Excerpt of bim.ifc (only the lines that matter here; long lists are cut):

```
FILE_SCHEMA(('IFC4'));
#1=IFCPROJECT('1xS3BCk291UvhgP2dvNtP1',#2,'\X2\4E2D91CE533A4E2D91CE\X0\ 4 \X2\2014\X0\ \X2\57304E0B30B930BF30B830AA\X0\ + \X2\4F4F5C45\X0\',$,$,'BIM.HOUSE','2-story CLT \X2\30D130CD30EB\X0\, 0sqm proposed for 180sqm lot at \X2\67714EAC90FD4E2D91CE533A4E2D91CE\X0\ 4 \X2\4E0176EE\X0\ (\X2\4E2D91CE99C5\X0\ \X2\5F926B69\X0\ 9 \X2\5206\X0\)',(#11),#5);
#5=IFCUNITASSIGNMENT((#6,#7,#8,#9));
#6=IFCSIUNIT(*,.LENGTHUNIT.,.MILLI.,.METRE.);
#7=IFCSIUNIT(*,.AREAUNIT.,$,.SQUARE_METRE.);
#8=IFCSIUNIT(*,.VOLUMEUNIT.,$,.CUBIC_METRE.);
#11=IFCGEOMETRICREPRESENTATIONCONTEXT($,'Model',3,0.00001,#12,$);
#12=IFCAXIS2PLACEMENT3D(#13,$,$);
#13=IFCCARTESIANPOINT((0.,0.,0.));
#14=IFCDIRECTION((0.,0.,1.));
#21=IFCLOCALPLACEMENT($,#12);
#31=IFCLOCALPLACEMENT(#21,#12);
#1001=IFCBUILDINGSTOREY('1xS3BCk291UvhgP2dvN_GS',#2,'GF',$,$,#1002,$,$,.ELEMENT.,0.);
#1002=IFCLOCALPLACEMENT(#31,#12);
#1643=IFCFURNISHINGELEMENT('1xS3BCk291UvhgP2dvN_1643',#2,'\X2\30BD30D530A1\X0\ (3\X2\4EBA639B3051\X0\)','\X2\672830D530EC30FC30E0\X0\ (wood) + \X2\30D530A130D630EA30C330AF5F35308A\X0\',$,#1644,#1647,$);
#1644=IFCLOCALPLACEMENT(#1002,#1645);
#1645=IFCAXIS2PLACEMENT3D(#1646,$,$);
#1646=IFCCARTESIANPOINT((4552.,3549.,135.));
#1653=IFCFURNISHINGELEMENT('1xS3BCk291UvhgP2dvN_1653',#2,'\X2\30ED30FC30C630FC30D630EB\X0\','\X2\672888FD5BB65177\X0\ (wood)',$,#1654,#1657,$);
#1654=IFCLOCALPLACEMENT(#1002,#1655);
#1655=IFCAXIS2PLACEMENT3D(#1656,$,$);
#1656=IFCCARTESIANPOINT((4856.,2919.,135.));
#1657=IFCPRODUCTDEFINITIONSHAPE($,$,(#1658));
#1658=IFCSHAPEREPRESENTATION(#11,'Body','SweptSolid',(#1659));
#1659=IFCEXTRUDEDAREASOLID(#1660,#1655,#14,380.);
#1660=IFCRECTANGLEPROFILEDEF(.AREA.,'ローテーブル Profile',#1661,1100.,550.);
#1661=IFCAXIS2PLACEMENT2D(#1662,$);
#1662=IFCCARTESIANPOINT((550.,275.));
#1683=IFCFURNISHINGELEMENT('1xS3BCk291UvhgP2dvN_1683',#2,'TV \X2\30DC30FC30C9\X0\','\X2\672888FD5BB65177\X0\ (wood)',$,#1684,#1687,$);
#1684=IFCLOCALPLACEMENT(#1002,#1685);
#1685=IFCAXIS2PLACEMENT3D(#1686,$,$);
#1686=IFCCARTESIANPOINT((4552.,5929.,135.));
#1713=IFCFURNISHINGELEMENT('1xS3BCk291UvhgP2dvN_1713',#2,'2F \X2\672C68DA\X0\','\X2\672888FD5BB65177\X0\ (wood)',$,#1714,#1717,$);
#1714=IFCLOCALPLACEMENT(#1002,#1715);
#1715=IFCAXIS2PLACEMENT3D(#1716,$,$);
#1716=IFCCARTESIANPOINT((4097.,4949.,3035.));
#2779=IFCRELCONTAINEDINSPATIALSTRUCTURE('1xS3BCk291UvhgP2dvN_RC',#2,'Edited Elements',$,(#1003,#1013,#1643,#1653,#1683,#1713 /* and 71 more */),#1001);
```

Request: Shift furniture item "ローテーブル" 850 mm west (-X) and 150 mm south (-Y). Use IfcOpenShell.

```python
import ifcopenshell
import ifcopenshell.api.geometry
import ifcopenshell.util.placement
import ifcopenshell.util.unit

model = ifcopenshell.open("bim.ifc")
unit_scale = ifcopenshell.util.unit.calculate_unit_scale(model)

item = model.by_guid("1xS3BCk291UvhgP2dvN_1653")
matrix = ifcopenshell.util.placement.get_local_placement(item.ObjectPlacement)
matrix[0, 3] -= 0.85 / unit_scale
matrix[1, 3] -= 0.15 / unit_scale
ifcopenshell.api.geometry.edit_object_placement(model, product=item, matrix=matrix, is_si=False)

print(ifcopenshell.util.placement.get_local_placement(item.ObjectPlacement).round(3) + 0.0)

model.write("bim_edited.ifc")
```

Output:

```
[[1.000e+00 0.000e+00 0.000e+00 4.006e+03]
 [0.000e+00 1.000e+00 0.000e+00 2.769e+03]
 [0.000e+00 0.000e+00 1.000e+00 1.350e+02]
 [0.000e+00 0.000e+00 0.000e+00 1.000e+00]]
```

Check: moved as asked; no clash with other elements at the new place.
